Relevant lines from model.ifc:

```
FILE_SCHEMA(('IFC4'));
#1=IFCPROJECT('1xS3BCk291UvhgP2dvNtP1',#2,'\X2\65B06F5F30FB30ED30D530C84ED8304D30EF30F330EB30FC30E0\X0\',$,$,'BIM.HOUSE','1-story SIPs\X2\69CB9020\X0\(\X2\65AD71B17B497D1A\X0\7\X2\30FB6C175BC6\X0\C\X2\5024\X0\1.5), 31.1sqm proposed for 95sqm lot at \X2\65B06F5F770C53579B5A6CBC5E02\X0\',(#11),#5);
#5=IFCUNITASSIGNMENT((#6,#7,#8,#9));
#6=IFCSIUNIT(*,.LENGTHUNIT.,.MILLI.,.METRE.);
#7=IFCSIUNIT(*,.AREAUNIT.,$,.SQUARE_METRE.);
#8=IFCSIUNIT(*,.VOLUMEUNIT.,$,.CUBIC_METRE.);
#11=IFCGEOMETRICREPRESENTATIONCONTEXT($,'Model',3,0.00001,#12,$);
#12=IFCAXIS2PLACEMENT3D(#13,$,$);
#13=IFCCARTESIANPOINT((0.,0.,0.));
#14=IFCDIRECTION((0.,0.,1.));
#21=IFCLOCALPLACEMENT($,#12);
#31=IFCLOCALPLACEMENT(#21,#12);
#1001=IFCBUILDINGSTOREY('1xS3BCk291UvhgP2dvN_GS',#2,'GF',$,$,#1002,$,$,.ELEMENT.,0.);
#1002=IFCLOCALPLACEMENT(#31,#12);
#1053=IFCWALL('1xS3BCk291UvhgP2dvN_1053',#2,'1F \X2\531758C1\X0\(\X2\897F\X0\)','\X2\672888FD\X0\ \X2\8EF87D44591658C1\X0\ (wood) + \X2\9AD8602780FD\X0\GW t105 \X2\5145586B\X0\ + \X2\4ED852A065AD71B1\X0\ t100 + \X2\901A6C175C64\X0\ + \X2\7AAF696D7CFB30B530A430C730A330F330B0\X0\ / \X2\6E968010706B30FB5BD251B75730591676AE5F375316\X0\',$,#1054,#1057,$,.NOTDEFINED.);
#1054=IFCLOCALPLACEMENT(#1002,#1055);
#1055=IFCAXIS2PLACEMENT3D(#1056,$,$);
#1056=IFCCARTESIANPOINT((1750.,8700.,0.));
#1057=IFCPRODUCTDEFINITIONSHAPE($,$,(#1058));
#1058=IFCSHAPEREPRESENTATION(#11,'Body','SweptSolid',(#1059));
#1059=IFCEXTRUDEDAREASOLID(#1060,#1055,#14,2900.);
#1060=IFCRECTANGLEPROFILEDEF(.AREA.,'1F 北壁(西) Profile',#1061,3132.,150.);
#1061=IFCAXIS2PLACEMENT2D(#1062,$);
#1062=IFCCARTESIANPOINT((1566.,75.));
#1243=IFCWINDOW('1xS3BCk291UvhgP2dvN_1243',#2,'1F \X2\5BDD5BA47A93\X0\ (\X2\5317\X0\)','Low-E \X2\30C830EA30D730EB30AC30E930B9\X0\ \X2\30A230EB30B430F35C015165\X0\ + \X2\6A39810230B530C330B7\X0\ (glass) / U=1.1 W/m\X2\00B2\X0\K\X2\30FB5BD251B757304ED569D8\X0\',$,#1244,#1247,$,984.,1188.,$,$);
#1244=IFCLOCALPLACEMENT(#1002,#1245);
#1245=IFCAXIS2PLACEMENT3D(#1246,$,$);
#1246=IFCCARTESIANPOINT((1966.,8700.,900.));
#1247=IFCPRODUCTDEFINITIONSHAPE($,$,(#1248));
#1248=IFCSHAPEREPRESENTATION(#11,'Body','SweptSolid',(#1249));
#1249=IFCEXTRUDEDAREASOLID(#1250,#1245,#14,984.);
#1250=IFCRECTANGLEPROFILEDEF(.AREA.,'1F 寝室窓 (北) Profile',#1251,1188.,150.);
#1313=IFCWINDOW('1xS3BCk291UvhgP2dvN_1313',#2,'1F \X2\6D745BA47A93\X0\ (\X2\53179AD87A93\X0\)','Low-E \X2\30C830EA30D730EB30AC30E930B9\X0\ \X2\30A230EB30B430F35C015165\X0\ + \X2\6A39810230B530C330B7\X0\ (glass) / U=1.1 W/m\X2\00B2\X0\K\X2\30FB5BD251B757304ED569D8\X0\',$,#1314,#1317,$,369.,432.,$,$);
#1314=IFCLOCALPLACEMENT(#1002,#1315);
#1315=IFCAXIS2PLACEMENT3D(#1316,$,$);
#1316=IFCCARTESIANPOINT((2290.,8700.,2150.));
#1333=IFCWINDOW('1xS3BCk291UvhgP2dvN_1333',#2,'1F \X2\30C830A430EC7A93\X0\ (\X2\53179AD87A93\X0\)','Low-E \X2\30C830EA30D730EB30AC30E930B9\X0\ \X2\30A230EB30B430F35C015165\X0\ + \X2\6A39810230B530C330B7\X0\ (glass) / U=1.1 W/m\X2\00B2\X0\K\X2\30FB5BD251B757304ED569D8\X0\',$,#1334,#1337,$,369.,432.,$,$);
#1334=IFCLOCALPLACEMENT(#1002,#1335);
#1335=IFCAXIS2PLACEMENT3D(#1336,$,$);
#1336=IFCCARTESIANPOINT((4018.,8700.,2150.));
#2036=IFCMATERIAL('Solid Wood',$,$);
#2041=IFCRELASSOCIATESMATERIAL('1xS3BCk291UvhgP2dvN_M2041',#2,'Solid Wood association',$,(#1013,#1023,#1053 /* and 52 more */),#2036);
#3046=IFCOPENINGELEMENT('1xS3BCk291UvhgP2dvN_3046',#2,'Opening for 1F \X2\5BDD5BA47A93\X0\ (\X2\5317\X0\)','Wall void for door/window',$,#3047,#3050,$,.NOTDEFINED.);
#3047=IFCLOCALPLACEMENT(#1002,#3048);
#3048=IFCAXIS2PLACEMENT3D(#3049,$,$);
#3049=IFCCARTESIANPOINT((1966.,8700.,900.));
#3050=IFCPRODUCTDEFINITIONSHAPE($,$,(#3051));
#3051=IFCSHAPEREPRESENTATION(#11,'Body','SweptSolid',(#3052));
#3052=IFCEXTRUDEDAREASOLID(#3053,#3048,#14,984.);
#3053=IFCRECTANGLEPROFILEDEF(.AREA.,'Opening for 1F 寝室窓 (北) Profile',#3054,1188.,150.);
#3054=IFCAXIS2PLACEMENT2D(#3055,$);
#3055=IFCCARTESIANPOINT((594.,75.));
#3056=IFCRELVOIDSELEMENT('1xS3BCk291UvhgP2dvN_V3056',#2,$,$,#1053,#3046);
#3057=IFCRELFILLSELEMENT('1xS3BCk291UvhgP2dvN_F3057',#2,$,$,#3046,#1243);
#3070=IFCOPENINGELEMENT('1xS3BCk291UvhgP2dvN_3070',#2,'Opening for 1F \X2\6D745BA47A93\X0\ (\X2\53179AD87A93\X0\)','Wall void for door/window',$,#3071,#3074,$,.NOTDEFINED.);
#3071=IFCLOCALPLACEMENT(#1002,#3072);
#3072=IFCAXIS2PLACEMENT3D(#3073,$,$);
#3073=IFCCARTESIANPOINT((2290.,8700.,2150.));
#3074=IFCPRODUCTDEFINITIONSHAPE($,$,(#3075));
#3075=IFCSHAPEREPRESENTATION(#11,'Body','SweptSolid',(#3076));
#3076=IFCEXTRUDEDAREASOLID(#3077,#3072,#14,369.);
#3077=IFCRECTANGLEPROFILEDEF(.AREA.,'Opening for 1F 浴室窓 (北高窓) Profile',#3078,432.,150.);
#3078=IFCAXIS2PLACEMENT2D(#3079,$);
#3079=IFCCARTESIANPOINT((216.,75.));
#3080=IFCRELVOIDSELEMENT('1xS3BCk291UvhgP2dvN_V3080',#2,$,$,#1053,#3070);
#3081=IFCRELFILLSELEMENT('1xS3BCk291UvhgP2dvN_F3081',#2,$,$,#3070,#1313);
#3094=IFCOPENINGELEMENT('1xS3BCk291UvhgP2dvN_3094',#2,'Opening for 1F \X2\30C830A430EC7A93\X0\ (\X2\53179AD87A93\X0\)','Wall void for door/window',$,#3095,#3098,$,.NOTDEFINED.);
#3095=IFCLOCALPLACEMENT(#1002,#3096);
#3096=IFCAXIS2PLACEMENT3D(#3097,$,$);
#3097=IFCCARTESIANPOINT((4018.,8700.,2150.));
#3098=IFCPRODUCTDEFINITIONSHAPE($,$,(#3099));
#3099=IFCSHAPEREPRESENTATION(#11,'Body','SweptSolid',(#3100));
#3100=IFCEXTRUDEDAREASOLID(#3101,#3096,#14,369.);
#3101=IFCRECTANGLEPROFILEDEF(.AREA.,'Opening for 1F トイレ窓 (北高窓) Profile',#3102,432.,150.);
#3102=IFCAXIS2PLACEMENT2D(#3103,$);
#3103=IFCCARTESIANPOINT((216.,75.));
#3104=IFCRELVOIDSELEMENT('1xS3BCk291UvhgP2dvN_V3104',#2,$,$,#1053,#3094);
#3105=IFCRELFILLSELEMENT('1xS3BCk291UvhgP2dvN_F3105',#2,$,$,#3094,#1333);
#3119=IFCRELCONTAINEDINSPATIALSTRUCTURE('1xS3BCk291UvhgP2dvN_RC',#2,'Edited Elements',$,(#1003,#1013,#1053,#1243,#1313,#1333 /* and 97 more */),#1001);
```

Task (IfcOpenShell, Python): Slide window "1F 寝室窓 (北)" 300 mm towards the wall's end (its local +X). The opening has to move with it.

```python
import ifcopenshell
import ifcopenshell.api.geometry
import ifcopenshell.util.placement

model = ifcopenshell.open("model.ifc")

window = model.by_guid("1xS3BCk291UvhgP2dvN_1243")
opening = window.FillsVoids[0].RelatingOpeningElement
wall = opening.VoidsElements[0].RelatingBuildingElement

wall_matrix = ifcopenshell.util.placement.get_local_placement(wall.ObjectPlacement)
shift = wall_matrix[:3, 0] * 300.0
before = ifcopenshell.util.placement.get_local_placement(window.ObjectPlacement)[:3, 3].copy()

# The window is not placed relative to its opening, so move both.
for product in (opening, window):
    matrix = ifcopenshell.util.placement.get_local_placement(product.ObjectPlacement)
    matrix[:3, 3] += shift
    ifcopenshell.api.geometry.edit_object_placement(model, product=product, matrix=matrix, is_si=False)

after = ifcopenshell.util.placement.get_local_placement(window.ObjectPlacement)[:3, 3]
print("window moved by", (after - before).round(3) + 0.0)

model.write("model_v2.ifc")
```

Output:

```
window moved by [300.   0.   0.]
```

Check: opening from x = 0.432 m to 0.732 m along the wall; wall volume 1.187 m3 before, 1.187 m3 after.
